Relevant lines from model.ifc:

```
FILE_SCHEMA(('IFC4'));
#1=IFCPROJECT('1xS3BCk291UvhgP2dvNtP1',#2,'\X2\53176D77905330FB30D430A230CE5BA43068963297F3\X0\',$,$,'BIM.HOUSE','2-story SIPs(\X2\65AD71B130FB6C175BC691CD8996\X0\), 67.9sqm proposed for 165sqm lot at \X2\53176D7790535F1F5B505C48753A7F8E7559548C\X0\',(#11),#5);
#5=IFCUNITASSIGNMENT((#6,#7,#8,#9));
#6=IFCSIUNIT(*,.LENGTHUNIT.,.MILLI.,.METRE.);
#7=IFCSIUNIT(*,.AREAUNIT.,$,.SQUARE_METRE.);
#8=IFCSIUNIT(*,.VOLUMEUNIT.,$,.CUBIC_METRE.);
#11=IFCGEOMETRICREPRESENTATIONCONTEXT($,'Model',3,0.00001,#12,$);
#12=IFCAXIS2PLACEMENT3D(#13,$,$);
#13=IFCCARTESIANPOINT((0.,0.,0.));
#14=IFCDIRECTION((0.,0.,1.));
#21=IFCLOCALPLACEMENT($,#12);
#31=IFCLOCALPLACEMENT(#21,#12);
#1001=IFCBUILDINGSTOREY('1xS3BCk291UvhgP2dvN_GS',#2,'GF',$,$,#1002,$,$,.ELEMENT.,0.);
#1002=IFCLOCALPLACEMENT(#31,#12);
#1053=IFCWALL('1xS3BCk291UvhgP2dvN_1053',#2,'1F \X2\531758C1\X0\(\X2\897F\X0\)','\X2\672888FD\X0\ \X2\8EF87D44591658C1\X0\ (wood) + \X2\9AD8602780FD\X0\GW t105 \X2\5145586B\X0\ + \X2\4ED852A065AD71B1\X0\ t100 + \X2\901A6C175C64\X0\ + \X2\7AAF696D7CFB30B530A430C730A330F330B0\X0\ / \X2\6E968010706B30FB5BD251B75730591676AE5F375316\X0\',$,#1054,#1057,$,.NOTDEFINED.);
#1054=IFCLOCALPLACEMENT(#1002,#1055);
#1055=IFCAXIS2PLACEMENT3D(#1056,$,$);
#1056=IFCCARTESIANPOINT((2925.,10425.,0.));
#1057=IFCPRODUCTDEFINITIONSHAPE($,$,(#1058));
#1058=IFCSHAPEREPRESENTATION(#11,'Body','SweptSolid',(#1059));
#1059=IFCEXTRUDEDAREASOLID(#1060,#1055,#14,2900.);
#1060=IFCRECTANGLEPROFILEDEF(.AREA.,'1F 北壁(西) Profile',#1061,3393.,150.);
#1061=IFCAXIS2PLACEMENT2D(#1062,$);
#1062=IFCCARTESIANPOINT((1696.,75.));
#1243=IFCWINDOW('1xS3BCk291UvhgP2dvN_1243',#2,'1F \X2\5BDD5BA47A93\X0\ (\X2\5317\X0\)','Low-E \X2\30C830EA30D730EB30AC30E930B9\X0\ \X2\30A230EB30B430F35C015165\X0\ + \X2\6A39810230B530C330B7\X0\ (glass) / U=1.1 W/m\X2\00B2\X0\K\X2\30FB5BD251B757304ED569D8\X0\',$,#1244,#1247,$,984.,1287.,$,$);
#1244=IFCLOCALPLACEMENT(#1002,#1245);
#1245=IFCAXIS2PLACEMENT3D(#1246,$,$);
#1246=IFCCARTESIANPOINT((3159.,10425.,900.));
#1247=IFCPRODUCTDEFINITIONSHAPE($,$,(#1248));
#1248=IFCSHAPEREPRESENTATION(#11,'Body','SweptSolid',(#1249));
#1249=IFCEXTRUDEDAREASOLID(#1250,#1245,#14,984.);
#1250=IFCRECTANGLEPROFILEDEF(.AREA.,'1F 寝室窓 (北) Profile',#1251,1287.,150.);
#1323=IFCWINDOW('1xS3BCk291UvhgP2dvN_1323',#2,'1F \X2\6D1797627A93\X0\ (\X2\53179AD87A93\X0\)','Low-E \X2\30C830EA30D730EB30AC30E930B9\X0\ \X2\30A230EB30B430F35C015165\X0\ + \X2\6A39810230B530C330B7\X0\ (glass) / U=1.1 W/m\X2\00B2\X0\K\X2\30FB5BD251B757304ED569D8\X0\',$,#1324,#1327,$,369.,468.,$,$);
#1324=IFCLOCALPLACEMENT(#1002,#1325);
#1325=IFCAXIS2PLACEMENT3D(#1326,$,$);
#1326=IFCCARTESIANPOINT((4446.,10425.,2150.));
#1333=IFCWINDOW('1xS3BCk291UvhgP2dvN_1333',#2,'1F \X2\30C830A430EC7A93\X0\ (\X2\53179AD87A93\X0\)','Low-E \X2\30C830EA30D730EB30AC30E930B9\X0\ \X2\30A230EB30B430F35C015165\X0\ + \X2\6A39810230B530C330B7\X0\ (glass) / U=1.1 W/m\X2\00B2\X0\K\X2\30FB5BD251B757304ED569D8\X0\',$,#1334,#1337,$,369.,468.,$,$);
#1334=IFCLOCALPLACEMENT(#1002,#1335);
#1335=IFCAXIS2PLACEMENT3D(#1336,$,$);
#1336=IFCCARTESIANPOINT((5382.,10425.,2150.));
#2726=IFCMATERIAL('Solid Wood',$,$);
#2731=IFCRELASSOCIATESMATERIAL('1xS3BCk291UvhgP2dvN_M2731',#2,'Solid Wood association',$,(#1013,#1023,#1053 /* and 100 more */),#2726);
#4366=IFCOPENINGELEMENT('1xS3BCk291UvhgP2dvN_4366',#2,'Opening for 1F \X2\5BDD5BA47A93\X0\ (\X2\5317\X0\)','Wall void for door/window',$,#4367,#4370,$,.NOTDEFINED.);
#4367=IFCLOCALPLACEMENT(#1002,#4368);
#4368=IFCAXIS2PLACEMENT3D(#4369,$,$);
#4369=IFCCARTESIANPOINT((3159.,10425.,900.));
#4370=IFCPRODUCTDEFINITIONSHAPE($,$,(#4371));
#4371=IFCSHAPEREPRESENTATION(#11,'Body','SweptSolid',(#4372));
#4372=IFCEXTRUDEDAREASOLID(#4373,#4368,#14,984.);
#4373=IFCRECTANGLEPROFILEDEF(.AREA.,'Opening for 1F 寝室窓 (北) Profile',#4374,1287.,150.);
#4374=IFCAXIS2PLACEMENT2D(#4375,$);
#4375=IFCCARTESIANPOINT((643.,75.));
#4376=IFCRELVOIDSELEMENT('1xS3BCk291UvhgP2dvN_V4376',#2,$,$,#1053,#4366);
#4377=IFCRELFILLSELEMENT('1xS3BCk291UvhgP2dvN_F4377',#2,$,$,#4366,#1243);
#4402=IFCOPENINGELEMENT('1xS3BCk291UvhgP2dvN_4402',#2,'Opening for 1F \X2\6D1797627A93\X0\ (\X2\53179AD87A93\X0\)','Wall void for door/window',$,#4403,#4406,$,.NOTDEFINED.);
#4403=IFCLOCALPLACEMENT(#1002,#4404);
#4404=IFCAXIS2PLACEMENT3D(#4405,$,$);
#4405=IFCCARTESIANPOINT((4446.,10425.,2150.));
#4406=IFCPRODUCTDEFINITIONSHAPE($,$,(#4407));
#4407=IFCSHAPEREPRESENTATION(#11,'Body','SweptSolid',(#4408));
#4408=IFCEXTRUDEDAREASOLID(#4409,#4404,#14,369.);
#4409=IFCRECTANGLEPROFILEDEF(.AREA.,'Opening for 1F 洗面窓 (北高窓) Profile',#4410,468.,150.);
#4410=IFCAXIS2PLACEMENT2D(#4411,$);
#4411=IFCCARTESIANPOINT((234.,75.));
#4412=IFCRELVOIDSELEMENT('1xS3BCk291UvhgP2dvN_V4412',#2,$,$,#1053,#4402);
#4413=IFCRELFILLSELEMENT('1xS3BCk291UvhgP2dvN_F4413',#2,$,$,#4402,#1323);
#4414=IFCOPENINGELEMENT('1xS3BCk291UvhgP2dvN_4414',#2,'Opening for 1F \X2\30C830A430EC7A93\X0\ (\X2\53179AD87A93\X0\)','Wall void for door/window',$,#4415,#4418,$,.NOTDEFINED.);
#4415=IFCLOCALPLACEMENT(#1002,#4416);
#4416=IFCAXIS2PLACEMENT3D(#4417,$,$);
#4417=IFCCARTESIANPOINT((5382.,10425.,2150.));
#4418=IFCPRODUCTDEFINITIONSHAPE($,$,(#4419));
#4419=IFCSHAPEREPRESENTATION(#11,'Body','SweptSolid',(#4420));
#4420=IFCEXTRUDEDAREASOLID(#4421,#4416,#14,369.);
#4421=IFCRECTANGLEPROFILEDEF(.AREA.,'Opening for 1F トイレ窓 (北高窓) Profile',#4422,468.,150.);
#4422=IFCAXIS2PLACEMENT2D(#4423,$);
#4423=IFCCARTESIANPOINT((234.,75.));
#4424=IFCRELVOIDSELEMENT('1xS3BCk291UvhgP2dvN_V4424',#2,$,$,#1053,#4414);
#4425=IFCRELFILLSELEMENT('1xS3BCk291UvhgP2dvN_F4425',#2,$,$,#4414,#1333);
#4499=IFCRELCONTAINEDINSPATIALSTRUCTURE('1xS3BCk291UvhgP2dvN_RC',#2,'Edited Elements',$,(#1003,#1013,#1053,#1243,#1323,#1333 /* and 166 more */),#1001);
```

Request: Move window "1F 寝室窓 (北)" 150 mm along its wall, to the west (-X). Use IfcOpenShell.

```python
import ifcopenshell
import ifcopenshell.api.geometry
import ifcopenshell.util.placement
import ifcopenshell.util.unit

model = ifcopenshell.open("model.ifc")
unit_scale = ifcopenshell.util.unit.calculate_unit_scale(model)

window = model.by_guid("1xS3BCk291UvhgP2dvN_1243")
opening = window.FillsVoids[0].RelatingOpeningElement
wall = opening.VoidsElements[0].RelatingBuildingElement

wall_matrix = ifcopenshell.util.placement.get_local_placement(wall.ObjectPlacement)
shift = wall_matrix[:3, 0] * -0.15 / unit_scale
before = ifcopenshell.util.placement.get_local_placement(window.ObjectPlacement)[:3, 3].copy()

# The window is not placed relative to its opening, so move both.
for product in (opening, window):
    matrix = ifcopenshell.util.placement.get_local_placement(product.ObjectPlacement)
    matrix[:3, 3] += shift
    ifcopenshell.api.geometry.edit_object_placement(model, product=product, matrix=matrix, is_si=False)

after = ifcopenshell.util.placement.get_local_placement(window.ObjectPlacement)[:3, 3]
print("window moved by", (after - before).round(3) + 0.0)

model.write("model_updated.ifc")
```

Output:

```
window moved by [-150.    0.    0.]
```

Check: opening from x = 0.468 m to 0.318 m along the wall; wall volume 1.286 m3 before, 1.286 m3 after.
